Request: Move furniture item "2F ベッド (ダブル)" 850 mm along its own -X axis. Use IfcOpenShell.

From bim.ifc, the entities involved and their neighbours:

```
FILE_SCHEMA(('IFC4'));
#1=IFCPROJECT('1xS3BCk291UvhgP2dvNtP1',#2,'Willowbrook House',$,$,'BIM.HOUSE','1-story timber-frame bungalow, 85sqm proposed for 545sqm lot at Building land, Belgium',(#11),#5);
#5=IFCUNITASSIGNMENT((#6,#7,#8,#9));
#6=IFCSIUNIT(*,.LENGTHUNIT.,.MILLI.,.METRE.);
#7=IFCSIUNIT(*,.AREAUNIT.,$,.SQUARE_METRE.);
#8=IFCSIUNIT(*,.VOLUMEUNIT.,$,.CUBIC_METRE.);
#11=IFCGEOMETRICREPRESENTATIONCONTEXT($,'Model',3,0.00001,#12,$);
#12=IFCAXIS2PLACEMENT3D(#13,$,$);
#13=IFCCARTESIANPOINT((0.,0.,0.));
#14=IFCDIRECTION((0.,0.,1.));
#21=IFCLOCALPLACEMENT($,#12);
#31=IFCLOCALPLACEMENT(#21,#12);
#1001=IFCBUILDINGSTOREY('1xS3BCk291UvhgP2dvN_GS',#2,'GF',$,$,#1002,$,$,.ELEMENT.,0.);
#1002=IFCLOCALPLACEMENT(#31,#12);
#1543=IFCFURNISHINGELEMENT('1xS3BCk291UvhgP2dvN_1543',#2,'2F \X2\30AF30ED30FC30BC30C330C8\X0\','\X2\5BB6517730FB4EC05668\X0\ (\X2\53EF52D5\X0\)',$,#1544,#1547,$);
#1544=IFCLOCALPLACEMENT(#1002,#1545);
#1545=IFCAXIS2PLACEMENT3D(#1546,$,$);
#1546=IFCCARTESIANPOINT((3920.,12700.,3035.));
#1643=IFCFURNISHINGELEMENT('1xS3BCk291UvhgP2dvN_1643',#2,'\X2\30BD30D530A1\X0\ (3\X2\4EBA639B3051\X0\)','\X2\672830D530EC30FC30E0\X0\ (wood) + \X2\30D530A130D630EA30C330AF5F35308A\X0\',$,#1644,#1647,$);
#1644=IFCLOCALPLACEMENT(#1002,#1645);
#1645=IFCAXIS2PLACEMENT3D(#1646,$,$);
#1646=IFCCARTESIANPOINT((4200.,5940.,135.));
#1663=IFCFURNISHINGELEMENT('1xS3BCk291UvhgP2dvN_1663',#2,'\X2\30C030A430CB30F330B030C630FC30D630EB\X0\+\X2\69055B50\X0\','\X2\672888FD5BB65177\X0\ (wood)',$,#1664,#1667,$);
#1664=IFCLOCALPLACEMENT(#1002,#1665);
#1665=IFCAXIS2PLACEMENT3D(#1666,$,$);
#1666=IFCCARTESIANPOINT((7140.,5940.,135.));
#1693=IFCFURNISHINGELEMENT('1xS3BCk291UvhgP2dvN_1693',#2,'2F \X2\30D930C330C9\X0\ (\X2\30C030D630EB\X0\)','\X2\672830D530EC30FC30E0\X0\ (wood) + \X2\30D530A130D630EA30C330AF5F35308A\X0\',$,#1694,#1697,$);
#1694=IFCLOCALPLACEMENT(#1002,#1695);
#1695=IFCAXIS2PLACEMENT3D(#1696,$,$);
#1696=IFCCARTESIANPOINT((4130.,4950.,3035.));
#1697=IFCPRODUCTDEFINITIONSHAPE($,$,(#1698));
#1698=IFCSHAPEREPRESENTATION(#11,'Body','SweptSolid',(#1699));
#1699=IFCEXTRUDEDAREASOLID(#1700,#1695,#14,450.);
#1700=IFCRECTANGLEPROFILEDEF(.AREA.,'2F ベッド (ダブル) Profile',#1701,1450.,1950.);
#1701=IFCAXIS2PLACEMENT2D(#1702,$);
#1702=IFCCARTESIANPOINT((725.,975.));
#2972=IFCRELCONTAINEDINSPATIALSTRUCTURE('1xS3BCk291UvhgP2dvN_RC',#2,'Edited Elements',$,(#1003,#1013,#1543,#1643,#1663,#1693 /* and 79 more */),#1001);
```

```python
import ifcopenshell
import ifcopenshell.api.geometry
import ifcopenshell.util.placement
import ifcopenshell.util.unit

model = ifcopenshell.open("bim.ifc")
unit_scale = ifcopenshell.util.unit.calculate_unit_scale(model)

item = model.by_guid("1xS3BCk291UvhgP2dvN_1693")
matrix = ifcopenshell.util.placement.get_local_placement(item.ObjectPlacement)
matrix[:3, 3] -= matrix[:3, 0] * 0.85 / unit_scale
ifcopenshell.api.geometry.edit_object_placement(model, product=item, matrix=matrix, is_si=False)

print(ifcopenshell.util.placement.get_local_placement(item.ObjectPlacement).round(3) + 0.0)

model.write("bim_edited.ifc")
```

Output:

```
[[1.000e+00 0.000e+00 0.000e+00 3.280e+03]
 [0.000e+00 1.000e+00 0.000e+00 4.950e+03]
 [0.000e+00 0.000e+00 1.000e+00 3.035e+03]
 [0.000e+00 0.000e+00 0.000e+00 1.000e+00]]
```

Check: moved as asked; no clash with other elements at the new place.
